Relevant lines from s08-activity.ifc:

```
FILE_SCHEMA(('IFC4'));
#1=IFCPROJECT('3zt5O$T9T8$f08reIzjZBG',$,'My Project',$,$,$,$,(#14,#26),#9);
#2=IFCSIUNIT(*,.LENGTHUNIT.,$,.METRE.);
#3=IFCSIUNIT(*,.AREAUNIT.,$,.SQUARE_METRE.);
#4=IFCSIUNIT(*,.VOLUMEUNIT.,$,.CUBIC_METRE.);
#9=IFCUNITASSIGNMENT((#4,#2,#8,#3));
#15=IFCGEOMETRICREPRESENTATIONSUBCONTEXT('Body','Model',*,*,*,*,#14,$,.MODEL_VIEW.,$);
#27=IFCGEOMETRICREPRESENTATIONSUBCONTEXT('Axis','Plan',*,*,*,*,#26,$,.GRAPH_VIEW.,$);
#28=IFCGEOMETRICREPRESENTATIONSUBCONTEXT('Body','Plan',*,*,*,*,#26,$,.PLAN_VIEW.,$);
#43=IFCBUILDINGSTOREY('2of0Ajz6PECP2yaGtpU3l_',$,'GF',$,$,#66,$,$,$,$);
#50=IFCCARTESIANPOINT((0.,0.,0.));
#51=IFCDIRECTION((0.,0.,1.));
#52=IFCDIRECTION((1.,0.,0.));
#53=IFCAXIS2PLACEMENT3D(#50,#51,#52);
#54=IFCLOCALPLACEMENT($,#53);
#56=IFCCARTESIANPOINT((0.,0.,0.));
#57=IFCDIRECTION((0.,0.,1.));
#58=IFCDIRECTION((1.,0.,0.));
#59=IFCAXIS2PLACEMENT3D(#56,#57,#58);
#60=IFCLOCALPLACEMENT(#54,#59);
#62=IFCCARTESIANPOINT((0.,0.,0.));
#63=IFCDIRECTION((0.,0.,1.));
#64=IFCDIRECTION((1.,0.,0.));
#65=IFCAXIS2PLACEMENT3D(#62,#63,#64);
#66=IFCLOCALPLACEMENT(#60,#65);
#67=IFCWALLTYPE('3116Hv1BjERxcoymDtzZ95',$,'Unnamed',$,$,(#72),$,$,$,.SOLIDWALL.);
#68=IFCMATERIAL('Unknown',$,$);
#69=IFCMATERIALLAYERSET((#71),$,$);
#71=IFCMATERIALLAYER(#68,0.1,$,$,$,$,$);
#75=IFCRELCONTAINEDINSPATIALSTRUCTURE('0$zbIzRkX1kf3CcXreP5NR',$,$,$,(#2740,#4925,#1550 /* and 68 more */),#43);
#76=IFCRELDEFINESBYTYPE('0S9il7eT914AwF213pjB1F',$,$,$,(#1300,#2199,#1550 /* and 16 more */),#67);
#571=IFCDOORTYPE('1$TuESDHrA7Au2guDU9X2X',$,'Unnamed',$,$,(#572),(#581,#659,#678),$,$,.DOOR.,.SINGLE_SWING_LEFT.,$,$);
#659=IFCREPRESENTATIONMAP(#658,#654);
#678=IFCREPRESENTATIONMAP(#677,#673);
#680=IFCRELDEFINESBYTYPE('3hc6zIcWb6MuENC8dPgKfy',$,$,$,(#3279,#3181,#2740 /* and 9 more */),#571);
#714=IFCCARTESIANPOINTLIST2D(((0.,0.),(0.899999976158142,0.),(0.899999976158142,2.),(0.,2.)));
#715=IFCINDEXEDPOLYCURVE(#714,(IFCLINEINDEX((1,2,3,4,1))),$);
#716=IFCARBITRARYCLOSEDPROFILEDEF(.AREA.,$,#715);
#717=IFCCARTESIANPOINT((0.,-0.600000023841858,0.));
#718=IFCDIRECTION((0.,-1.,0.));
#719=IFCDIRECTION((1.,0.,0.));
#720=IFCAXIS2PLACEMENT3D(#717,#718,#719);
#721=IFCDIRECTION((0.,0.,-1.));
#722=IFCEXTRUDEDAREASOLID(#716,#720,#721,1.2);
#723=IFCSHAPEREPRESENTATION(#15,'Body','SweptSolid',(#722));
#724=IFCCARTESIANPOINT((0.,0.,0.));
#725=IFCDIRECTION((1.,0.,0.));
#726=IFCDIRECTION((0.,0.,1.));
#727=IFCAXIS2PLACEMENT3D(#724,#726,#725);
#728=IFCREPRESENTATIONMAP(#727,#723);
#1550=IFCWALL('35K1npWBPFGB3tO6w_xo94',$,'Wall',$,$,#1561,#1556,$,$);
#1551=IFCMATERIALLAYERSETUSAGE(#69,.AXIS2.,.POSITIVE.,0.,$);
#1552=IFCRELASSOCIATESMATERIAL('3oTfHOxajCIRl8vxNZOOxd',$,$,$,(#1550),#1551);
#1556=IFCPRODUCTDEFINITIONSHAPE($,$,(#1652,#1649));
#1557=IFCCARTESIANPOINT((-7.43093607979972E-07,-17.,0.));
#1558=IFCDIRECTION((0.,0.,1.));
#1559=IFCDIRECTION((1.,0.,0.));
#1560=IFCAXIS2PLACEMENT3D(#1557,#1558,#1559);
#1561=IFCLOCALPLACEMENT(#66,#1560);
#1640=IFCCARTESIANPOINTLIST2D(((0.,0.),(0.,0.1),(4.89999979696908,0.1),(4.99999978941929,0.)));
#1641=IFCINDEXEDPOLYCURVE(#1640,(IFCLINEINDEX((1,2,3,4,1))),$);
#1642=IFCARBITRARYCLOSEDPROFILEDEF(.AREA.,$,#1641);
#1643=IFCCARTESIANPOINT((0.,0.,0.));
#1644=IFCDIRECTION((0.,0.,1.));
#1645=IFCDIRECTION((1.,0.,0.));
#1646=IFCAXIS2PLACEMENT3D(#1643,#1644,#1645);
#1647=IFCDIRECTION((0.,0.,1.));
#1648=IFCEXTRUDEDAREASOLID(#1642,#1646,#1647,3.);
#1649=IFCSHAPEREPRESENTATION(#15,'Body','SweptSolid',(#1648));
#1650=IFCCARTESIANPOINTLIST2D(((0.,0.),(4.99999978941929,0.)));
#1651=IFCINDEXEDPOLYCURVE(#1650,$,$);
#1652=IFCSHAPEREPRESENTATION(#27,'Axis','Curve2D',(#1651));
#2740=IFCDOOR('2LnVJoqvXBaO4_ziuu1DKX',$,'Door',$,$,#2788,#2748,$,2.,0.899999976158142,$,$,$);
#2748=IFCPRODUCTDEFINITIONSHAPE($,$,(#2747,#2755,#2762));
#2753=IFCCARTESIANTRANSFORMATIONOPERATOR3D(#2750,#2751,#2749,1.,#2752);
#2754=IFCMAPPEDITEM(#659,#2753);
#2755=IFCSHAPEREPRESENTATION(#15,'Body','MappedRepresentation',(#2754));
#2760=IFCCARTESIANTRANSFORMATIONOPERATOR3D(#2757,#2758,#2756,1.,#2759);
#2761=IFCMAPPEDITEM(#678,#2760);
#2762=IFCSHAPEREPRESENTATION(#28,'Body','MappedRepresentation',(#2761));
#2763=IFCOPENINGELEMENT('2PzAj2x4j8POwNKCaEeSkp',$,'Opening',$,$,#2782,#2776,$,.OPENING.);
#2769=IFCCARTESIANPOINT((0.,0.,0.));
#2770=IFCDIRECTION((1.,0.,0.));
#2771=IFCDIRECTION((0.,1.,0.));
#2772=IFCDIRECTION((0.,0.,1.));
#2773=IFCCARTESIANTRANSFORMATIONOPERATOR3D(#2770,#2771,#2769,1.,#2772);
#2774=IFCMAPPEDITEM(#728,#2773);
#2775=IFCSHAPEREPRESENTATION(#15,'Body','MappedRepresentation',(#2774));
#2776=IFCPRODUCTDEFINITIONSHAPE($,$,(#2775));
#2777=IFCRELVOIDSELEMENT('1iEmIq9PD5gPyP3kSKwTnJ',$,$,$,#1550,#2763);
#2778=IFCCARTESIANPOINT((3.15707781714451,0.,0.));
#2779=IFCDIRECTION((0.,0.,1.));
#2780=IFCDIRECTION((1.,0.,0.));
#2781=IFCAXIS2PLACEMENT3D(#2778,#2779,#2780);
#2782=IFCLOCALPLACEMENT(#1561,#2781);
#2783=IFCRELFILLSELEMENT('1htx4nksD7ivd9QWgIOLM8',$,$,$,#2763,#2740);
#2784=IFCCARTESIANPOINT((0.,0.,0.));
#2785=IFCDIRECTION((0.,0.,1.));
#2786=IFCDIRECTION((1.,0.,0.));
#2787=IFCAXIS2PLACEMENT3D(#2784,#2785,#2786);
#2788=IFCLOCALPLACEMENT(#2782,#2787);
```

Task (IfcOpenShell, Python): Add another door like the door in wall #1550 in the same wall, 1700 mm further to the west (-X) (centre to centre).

```python
import ifcopenshell
import ifcopenshell.api.feature
import ifcopenshell.api.geometry
import ifcopenshell.api.root
import ifcopenshell.geom
import ifcopenshell.util.element
import ifcopenshell.util.placement
import ifcopenshell.util.shape
import ifcopenshell.util.unit

model = ifcopenshell.open("s08-activity.ifc")
unit_scale = ifcopenshell.util.unit.calculate_unit_scale(model)
settings = ifcopenshell.geom.settings()


def volume(element):
    """Net volume in cubic metres, openings subtracted."""
    shape = ifcopenshell.geom.create_shape(settings, element)
    return ifcopenshell.util.shape.get_volume(shape.geometry)


door = model.by_guid("2LnVJoqvXBaO4_ziuu1DKX")
opening = door.FillsVoids[0].RelatingOpeningElement
wall = opening.VoidsElements[0].RelatingBuildingElement
before = volume(wall)
shift = ifcopenshell.util.placement.get_local_placement(wall.ObjectPlacement)[:3, 0] * -1.7 / unit_scale

# copy_class copies the void relationship, type, container and properties, but no geometry.
new_opening = ifcopenshell.api.root.copy_class(model, product=opening)
new_opening.Representation = ifcopenshell.util.element.copy_deep(
    model, opening.Representation, exclude=["IfcGeometricRepresentationContext", "IfcRepresentationMap"]
)
new_door = ifcopenshell.api.root.copy_class(model, product=door)
new_door.Representation = ifcopenshell.util.element.copy_deep(
    model, door.Representation, exclude=["IfcGeometricRepresentationContext", "IfcRepresentationMap"]
)
ifcopenshell.api.feature.add_filling(model, opening=new_opening, element=new_door)

for old, new in ((opening, new_opening), (door, new_door)):
    matrix = ifcopenshell.util.placement.get_local_placement(old.ObjectPlacement)
    matrix[:3, 3] += shift
    ifcopenshell.api.geometry.edit_object_placement(model, product=new, matrix=matrix, is_si=False)

after = volume(wall)

print(f"wall volume {before:.3f} -> {after:.3f} m3")

model.write("s08-activity_rev.ifc")
```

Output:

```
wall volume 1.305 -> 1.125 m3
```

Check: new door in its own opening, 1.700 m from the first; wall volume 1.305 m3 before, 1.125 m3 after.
